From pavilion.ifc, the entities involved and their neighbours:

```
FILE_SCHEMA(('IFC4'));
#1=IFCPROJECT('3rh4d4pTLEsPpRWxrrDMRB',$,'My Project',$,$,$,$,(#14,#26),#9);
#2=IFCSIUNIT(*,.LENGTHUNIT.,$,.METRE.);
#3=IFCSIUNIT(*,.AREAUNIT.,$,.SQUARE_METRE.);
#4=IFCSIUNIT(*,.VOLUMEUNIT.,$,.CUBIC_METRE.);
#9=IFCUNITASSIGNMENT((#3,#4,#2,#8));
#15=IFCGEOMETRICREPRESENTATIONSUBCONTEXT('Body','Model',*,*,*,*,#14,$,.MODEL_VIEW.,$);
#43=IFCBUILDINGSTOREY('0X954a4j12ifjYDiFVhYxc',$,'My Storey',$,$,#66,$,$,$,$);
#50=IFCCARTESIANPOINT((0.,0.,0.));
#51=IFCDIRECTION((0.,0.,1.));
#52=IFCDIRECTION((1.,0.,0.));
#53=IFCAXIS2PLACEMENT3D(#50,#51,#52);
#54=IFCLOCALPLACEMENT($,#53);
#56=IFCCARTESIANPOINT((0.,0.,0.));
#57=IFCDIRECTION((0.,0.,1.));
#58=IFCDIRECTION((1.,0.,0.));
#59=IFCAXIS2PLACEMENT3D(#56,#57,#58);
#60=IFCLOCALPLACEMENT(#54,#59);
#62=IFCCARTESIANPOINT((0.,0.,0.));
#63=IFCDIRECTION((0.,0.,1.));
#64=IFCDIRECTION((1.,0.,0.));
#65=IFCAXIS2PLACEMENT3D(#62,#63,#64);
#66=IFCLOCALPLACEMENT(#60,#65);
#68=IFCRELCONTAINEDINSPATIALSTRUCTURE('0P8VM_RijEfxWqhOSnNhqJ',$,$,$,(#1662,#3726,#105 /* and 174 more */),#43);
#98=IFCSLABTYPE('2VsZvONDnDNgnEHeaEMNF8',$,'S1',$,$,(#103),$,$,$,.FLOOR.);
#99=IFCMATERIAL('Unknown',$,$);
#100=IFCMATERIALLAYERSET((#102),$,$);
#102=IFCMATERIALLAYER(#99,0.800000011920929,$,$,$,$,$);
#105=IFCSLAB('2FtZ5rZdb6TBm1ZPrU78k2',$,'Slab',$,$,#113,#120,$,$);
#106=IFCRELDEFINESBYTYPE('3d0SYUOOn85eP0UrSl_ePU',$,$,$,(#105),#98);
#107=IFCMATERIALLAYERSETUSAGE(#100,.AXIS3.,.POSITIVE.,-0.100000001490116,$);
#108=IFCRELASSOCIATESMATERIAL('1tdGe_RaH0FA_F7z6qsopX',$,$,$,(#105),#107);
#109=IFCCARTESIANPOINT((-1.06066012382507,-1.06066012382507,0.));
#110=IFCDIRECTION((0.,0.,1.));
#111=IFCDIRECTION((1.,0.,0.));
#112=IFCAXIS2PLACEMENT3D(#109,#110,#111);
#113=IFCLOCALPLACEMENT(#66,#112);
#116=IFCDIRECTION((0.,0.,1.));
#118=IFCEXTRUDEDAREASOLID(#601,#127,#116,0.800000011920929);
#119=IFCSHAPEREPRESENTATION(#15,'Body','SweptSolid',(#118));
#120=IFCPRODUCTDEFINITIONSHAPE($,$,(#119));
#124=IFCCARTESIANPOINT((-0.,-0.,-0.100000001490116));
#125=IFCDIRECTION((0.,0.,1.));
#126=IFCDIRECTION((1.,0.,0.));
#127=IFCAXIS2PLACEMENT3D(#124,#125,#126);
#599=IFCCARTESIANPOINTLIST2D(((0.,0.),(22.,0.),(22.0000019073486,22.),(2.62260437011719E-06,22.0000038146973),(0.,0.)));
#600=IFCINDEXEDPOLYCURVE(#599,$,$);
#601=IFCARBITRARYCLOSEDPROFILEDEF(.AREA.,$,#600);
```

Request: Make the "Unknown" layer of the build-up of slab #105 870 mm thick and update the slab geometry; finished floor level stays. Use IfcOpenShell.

```python
import ifcopenshell
import ifcopenshell.util.element
import ifcopenshell.util.representation

model = ifcopenshell.open("pavilion.ifc")

layer_set = model.by_id(100)
layer = next(l for l in layer_set.MaterialLayers if l.Material and l.Material.Name == "Unknown")
change = 0.87 - layer.LayerThickness
layer.LayerThickness += change

# Geometry does not follow the layer set by itself.
slabs = [e for e in ifcopenshell.util.element.get_elements_by_material(model, layer_set) if e.is_a("IfcSlab")]
for slab in sorted(slabs, key=lambda e: e.id()):
    body = ifcopenshell.util.representation.get_representation(slab, "Model", "Body")
    solid = body.Items[0]
    old_depth = solid.Depth
    solid.Depth += change
    # Extruded upwards: lower the start of the extrusion so the top stays.
    x, y, z = solid.Position.Location.Coordinates
    solid.Position.Location = model.createIfcCartesianPoint((x, y, z - change))
    print(slab.id(), f"{old_depth:g} -> {solid.Depth:g}")

# The layers are counted up from the underside, which has moved.
for usage in {ifcopenshell.util.element.get_material(slab) for slab in slabs}:
    usage.OffsetFromReferenceLine -= change

model.write("pavilion-out.ifc")
```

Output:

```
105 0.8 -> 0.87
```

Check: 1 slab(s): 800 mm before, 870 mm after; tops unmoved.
